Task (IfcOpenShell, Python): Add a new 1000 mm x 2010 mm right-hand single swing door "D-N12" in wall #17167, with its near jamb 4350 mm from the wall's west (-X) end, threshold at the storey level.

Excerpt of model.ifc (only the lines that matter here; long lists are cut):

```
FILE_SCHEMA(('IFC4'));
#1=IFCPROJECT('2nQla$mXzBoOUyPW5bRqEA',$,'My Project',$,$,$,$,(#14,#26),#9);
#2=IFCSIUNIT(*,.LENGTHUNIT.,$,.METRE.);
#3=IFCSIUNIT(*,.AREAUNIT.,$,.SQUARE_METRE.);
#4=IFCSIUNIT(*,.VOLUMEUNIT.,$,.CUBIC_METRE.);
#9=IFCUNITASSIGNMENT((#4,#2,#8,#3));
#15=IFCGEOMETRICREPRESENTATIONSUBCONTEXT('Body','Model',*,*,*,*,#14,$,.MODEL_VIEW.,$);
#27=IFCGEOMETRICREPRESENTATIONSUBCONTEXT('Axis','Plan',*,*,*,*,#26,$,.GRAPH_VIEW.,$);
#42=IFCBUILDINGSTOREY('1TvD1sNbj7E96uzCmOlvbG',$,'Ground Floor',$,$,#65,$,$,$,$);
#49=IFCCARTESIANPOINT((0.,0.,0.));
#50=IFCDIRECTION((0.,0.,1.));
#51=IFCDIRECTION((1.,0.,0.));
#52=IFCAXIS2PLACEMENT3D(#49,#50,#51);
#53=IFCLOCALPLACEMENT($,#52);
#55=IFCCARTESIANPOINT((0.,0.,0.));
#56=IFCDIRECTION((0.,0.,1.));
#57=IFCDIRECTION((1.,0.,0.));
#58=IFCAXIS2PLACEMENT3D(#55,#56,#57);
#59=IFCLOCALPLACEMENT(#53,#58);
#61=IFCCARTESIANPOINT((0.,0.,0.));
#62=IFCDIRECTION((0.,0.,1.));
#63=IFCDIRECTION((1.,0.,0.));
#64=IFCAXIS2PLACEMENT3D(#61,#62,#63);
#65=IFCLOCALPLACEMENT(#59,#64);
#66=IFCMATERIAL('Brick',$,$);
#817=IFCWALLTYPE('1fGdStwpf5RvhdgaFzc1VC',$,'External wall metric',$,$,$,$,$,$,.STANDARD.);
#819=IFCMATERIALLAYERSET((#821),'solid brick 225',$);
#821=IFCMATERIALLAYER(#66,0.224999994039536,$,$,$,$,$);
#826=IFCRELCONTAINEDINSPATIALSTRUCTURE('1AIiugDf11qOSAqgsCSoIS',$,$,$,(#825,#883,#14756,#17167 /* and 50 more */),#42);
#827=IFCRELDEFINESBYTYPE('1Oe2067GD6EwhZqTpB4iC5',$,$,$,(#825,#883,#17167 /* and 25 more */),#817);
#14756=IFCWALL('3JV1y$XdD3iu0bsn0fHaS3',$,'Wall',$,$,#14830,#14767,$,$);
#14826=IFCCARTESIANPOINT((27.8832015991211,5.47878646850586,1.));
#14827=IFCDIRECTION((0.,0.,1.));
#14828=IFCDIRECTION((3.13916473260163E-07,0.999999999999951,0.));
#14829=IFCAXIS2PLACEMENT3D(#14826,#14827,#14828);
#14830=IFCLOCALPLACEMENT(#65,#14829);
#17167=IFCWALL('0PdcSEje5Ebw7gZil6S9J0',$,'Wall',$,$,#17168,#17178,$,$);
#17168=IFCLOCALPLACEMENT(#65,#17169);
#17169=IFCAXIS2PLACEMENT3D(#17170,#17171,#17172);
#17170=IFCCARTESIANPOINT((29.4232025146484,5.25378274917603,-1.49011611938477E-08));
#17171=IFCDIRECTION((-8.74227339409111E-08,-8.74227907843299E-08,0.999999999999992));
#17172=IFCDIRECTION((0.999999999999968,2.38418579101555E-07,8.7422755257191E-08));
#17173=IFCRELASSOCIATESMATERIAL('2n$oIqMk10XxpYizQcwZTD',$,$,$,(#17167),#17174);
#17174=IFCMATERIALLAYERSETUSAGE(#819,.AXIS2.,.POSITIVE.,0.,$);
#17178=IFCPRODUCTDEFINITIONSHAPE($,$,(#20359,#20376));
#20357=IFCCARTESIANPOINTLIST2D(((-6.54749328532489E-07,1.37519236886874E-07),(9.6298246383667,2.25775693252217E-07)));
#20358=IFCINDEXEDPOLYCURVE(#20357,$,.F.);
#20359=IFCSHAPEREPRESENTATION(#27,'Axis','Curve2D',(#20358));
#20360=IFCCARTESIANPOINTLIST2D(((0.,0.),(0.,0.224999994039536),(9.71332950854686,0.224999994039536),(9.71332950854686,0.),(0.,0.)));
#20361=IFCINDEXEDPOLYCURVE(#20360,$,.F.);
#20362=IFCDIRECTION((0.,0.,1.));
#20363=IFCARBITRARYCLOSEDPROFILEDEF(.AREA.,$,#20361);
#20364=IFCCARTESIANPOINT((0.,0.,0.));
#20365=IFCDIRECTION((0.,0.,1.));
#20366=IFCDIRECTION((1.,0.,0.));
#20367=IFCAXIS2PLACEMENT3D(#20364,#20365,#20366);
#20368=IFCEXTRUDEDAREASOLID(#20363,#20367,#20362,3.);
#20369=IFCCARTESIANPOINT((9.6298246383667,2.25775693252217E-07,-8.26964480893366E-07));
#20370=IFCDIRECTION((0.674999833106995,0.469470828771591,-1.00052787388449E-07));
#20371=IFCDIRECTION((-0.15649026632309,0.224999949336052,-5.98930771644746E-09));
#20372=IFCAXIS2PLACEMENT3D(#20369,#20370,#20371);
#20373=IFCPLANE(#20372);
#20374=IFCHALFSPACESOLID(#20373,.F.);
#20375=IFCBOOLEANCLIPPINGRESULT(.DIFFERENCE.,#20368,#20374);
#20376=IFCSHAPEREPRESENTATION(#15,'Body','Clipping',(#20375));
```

```python
import numpy as np
import ifcopenshell
import ifcopenshell.api.feature
import ifcopenshell.api.geometry
import ifcopenshell.api.root
import ifcopenshell.api.spatial
import ifcopenshell.geom
import ifcopenshell.util.element
import ifcopenshell.util.placement
import ifcopenshell.util.representation
import ifcopenshell.util.shape
import ifcopenshell.util.unit

model = ifcopenshell.open("model.ifc")
unit_scale = ifcopenshell.util.unit.calculate_unit_scale(model)
settings = ifcopenshell.geom.settings()


def volume(element):
    """Net volume in cubic metres, openings subtracted."""
    shape = ifcopenshell.geom.create_shape(settings, element)
    return ifcopenshell.util.shape.get_volume(shape.geometry)


wall = model.by_guid("0PdcSEje5Ebw7gZil6S9J0")
storey = ifcopenshell.util.element.get_container(wall, ifc_class="IfcBuildingStorey")
context = ifcopenshell.util.representation.get_context(model, "Model", "Body", "MODEL_VIEW")
before = volume(wall)

width, height, from_end, sill = 1, 2.01, 4.35, 0.0  # metres

# The wall runs along its own X axis, and the end named is its -X end.
wall_shape = ifcopenshell.geom.create_shape(settings, wall)
x, y, z = ifcopenshell.util.shape.get_vertices(wall_shape.geometry).T
start = x.min() + from_end
face, thickness = float(y.min()), float(y.max() - y.min())
wall_matrix = ifcopenshell.util.placement.get_local_placement(wall.ObjectPlacement)
level = ifcopenshell.util.placement.get_local_placement(storey.ObjectPlacement)[2, 3]


def in_wall(x, y):
    """Placement at x, y metres in the wall's axes, at sill height."""
    matrix = wall_matrix.copy()
    matrix[:, 3] = wall_matrix @ np.array([x / unit_scale, y / unit_scale, 0.0, 1.0])
    matrix[2, 3] = level + sill / unit_scale
    return matrix


# Opening: a box that overshoots both wall faces by 50 mm.
opening = ifcopenshell.api.root.create_entity(model, ifc_class="IfcOpeningElement", predefined_type="OPENING")
box = ifcopenshell.api.geometry.add_wall_representation(
    model, context=context, length=width, height=height, thickness=thickness + 0.1
)
ifcopenshell.api.geometry.assign_representation(model, product=opening, representation=box)
ifcopenshell.api.geometry.edit_object_placement(model, product=opening, matrix=in_wall(start, face - 0.05), is_si=False)
ifcopenshell.api.feature.add_feature(model, feature=opening, element=wall)

door = ifcopenshell.api.root.create_entity(model, ifc_class="IfcDoor", name="D-N12", predefined_type="DOOR")
door.OverallWidth, door.OverallHeight = width / unit_scale, height / unit_scale
door.OperationType = "SINGLE_SWING_RIGHT"
body = ifcopenshell.api.geometry.add_door_representation(
    model,
    context=context,
    overall_width=door.OverallWidth,
    overall_height=door.OverallHeight,
    operation_type="SINGLE_SWING_RIGHT",
    lining_properties={"LiningDepth": thickness / unit_scale, "ThresholdDepth": thickness / unit_scale},
)
ifcopenshell.api.geometry.assign_representation(model, product=door, representation=body)
ifcopenshell.api.spatial.assign_container(model, products=[door], relating_structure=storey)
ifcopenshell.api.feature.add_filling(model, opening=opening, element=door)

# The lining spans the wall, so the door starts at the wall face.
ifcopenshell.api.geometry.edit_object_placement(model, product=door, matrix=in_wall(start, face), is_si=False)

after = volume(wall)

print(f"wall volume {before:.3f} -> {after:.3f} m3")

model.write("model_v2.ifc")
```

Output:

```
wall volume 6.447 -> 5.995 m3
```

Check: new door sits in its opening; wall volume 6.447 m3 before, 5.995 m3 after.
